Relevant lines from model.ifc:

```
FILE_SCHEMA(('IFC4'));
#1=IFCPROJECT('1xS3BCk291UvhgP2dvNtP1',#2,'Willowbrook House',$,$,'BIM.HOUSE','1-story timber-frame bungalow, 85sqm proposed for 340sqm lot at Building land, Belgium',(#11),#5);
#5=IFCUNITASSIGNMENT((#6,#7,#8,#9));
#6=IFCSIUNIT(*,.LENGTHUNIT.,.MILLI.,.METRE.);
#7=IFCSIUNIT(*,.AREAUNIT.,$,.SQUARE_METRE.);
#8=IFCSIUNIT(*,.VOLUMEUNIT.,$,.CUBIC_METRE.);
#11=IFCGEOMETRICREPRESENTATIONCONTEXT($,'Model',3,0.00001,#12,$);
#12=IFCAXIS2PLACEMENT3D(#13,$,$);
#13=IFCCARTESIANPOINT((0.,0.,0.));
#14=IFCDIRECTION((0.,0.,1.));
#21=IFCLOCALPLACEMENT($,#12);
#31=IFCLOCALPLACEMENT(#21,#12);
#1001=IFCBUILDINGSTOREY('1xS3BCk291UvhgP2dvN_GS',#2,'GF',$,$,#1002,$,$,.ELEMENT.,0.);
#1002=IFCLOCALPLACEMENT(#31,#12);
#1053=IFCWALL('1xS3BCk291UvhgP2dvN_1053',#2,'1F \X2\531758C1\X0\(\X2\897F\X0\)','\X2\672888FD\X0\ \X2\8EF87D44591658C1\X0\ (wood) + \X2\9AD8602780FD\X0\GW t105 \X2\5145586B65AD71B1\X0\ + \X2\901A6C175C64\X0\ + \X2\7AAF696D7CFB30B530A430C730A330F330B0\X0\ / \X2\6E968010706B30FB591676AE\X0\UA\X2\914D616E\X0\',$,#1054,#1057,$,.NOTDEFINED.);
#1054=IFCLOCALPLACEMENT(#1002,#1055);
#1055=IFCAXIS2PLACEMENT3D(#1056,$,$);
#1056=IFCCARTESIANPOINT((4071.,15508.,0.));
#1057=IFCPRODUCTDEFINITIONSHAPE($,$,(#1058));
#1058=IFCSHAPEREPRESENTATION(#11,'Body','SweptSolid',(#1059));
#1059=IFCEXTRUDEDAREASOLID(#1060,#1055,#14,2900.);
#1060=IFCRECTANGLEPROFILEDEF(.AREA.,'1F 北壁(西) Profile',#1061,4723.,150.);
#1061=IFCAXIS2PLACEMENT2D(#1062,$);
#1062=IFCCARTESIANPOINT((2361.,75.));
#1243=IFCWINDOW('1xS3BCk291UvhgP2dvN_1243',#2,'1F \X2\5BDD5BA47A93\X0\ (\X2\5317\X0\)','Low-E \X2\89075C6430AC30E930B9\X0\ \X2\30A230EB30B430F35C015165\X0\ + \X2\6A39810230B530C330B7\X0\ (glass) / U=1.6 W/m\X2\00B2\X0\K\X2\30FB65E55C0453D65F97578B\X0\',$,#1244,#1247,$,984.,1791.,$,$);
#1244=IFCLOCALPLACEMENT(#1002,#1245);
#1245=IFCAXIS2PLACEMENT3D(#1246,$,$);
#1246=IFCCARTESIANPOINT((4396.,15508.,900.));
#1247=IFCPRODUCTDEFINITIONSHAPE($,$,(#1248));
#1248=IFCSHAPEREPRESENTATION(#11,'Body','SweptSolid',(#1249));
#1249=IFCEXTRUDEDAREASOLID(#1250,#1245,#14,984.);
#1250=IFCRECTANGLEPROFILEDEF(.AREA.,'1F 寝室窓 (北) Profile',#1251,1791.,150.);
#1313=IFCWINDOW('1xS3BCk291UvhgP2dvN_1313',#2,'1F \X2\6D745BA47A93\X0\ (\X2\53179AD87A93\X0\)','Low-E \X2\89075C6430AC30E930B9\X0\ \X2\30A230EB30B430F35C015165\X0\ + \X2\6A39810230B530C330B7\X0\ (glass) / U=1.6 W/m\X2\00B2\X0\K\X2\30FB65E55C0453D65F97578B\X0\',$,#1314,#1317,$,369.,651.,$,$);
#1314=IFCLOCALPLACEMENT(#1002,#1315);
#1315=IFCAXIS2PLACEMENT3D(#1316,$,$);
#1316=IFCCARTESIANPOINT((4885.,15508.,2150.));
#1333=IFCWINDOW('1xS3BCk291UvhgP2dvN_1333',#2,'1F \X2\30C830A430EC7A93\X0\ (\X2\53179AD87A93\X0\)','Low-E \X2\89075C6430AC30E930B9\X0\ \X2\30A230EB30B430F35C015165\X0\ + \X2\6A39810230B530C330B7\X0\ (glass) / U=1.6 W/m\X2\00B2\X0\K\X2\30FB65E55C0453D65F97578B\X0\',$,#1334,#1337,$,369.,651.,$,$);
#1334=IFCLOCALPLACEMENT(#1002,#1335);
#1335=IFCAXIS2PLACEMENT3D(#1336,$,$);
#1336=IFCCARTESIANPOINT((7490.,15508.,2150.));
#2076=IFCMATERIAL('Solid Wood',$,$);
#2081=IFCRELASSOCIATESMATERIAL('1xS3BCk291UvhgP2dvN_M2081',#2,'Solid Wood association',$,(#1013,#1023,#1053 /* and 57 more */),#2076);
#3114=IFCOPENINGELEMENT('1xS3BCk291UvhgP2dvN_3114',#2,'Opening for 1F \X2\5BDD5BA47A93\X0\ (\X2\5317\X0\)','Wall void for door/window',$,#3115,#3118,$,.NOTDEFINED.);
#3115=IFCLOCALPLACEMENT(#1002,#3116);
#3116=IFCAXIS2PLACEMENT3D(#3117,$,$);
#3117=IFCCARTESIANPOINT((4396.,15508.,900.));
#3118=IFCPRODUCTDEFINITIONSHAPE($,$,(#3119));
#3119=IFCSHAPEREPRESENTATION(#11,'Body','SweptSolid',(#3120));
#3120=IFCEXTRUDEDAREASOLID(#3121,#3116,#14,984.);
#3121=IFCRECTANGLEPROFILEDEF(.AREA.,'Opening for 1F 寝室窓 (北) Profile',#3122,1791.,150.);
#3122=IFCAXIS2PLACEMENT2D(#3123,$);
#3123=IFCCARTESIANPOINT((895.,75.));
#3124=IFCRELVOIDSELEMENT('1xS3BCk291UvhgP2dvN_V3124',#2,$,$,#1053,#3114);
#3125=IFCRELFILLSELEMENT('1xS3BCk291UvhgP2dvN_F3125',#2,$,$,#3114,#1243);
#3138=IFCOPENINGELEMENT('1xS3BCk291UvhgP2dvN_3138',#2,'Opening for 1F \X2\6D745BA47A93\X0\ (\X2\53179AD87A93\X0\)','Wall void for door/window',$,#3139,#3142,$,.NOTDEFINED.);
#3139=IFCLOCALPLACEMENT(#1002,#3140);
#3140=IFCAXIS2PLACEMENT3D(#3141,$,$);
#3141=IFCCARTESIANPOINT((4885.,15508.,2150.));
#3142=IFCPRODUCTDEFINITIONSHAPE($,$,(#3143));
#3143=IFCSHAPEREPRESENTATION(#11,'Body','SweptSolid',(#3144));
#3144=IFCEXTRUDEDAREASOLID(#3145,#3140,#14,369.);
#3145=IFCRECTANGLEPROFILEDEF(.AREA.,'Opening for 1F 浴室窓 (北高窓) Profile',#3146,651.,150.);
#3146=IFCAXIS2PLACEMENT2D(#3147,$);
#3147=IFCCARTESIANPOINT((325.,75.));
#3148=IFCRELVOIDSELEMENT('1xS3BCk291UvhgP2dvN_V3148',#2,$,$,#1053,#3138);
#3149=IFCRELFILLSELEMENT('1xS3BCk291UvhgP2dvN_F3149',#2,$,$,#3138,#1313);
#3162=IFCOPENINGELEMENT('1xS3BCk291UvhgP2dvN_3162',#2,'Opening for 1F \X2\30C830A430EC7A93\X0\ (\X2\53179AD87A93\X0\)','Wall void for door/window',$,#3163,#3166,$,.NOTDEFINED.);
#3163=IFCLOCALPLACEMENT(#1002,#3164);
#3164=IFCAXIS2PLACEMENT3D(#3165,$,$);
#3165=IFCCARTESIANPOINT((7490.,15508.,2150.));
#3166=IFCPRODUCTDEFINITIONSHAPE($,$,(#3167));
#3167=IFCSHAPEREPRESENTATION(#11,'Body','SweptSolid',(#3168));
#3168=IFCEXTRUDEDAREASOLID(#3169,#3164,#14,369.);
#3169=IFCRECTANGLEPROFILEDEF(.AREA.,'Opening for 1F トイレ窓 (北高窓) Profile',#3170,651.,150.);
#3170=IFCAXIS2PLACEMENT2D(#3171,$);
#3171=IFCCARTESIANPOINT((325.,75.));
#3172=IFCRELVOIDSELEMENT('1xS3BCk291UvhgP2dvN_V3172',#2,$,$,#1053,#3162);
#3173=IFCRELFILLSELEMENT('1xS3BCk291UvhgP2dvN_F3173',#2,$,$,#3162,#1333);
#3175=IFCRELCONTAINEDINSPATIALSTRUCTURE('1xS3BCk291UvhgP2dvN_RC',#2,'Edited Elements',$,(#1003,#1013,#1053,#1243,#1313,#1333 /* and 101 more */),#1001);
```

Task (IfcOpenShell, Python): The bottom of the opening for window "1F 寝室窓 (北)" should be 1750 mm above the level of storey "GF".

```python
import numpy as np
import ifcopenshell
import ifcopenshell.api.geometry
import ifcopenshell.geom
import ifcopenshell.util.element
import ifcopenshell.util.placement
import ifcopenshell.util.shape
import ifcopenshell.util.unit

model = ifcopenshell.open("model.ifc")
unit_scale = ifcopenshell.util.unit.calculate_unit_scale(model)

window = model.by_guid("1xS3BCk291UvhgP2dvN_1243")
opening = window.FillsVoids[0].RelatingOpeningElement
storey = ifcopenshell.util.element.get_container(window, ifc_class="IfcBuildingStorey")
level = ifcopenshell.util.placement.get_local_placement(storey.ObjectPlacement)[2, 3]

# The opening's origin need not be at the sill, so measure its lowest point.
shape = ifcopenshell.geom.create_shape(ifcopenshell.geom.settings(), opening)
bottom = ifcopenshell.util.shape.get_shape_bottom_elevation(shape, shape.geometry) / unit_scale
dz = level + 1750.0 - bottom

shift = np.array([0.0, 0.0, dz])
# The window is not placed relative to its opening, so move both.
for product in (opening, window):
    matrix = ifcopenshell.util.placement.get_local_placement(product.ObjectPlacement)
    matrix[:3, 3] += shift
    ifcopenshell.api.geometry.edit_object_placement(model, product=product, matrix=matrix, is_si=False)

print(f"moved by {dz * unit_scale:+.3f} m")

model.write("model-out.ifc")
```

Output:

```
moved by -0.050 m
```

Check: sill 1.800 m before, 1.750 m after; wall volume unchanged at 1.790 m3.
